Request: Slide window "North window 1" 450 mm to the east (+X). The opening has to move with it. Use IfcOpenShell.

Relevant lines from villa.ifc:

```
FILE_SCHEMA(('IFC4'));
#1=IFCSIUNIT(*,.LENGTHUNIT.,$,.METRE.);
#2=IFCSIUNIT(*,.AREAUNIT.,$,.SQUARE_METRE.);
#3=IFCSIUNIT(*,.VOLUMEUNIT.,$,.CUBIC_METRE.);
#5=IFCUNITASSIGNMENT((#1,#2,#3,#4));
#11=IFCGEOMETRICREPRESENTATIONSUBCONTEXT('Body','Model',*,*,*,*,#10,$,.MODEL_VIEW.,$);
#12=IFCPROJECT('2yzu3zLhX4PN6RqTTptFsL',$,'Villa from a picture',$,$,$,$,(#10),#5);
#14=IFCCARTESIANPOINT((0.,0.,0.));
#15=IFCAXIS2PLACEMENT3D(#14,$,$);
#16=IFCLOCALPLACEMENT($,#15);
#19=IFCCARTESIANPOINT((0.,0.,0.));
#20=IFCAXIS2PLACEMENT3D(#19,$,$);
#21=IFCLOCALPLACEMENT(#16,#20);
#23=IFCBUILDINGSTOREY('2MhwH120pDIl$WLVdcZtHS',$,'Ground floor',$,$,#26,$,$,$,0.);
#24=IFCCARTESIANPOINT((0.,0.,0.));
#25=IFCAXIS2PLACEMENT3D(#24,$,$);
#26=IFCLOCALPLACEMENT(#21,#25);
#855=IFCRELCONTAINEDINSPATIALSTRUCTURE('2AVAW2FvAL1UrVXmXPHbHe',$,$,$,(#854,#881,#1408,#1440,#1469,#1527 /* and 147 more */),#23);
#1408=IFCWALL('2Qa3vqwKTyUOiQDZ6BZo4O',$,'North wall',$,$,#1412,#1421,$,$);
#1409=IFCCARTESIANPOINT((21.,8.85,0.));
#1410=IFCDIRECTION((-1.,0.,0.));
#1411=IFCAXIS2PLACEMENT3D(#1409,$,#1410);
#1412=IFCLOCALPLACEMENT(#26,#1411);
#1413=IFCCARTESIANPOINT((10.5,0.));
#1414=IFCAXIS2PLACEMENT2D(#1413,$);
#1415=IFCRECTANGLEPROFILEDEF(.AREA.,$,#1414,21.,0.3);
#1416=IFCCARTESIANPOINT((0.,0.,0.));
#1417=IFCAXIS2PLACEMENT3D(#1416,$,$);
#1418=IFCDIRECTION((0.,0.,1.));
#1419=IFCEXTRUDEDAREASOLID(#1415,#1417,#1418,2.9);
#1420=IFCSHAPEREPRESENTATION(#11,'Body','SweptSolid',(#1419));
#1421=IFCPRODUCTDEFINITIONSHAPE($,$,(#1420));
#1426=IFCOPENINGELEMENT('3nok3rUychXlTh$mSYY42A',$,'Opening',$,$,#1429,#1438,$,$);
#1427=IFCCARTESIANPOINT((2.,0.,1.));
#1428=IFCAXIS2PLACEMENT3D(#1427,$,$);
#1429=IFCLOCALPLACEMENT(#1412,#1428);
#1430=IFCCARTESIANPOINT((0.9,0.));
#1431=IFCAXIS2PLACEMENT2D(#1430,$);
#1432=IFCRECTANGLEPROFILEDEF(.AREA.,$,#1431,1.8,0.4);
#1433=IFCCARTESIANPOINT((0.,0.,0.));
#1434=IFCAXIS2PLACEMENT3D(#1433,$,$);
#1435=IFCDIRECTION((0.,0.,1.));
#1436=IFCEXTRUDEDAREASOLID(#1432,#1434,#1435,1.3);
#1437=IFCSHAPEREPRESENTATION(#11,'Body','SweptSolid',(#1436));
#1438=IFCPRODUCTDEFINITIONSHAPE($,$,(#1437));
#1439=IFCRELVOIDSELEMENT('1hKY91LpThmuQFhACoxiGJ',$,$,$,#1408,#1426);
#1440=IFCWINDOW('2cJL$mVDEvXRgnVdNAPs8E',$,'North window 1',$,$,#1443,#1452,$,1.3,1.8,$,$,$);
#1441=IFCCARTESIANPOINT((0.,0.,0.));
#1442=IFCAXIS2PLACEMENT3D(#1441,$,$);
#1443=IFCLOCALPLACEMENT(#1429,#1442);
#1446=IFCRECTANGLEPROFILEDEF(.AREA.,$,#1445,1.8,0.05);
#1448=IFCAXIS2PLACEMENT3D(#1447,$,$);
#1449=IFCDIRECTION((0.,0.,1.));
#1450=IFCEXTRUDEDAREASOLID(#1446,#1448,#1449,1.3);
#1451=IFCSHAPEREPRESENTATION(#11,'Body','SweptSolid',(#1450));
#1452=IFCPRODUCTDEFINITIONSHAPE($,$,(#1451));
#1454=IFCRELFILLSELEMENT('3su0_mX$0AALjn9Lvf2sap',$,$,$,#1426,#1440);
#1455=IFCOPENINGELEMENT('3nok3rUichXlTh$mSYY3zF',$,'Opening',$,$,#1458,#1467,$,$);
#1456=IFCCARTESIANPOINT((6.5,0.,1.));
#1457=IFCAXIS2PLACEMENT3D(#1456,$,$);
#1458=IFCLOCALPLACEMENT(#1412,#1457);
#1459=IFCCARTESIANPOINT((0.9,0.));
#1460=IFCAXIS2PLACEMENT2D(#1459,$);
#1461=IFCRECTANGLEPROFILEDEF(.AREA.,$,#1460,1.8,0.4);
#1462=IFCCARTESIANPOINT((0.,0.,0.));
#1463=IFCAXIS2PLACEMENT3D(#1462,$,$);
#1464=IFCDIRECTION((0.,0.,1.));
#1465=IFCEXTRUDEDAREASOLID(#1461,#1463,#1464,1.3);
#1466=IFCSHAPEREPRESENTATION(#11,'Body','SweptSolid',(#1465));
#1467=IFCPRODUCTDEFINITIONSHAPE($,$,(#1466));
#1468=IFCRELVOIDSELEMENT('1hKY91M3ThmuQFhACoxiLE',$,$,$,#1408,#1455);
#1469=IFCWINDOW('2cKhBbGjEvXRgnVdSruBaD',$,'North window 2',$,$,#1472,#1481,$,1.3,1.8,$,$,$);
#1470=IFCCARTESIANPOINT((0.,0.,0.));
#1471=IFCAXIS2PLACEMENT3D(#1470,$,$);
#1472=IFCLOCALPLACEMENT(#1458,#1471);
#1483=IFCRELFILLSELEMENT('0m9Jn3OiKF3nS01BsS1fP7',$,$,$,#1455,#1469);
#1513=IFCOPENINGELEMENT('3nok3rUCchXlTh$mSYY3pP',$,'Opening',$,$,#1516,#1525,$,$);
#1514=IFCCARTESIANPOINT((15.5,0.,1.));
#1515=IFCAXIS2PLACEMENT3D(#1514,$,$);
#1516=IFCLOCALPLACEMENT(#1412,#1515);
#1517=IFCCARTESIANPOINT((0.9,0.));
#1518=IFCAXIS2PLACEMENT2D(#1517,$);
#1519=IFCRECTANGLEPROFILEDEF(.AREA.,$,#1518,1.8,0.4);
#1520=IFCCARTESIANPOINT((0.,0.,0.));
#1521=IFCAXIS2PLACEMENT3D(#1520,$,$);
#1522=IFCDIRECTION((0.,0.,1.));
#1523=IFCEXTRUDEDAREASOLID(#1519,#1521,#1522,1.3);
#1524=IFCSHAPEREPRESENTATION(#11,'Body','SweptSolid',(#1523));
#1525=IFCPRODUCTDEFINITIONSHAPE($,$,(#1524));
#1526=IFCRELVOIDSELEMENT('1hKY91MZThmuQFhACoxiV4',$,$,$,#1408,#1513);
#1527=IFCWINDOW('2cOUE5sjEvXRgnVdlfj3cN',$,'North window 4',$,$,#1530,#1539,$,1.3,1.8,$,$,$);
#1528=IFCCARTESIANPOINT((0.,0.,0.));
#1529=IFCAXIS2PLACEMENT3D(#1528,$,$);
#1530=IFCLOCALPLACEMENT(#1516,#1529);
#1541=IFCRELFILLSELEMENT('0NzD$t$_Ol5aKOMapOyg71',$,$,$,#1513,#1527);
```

```python
import ifcopenshell
import ifcopenshell.api.geometry
import ifcopenshell.util.placement

model = ifcopenshell.open("villa.ifc")

window = model.by_guid("2cJL$mVDEvXRgnVdNAPs8E")
opening = window.FillsVoids[0].RelatingOpeningElement
wall = opening.VoidsElements[0].RelatingBuildingElement

wall_matrix = ifcopenshell.util.placement.get_local_placement(wall.ObjectPlacement)
shift = wall_matrix[:3, 0] * -0.45
before = ifcopenshell.util.placement.get_local_placement(window.ObjectPlacement)[:3, 3].copy()

# The window is placed relative to its opening, so it follows when the opening moves.
matrix = ifcopenshell.util.placement.get_local_placement(opening.ObjectPlacement)
matrix[:3, 3] += shift
ifcopenshell.api.geometry.edit_object_placement(
    model, product=opening, matrix=matrix, is_si=False, should_transform_children=True
)

after = ifcopenshell.util.placement.get_local_placement(window.ObjectPlacement)[:3, 3]
print("window moved by", (after - before).round(3) + 0.0)

model.write("villa_v2.ifc")
```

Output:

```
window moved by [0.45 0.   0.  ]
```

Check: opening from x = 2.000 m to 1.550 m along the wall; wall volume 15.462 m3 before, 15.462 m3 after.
